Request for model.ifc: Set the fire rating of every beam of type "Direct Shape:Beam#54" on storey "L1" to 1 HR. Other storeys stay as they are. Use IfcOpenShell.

First a look at what the model holds.

```python
import ifcopenshell
import ifcopenshell.util.element

model = ifcopenshell.open("model.ifc")
print(model.schema)
storey = next(s for s in model.by_type("IfcBuildingStorey") if s.Name == "L1")
beams = [e for e in ifcopenshell.util.element.get_decomposition(storey) if e.is_a("IfcBeam")]
seen = {}
for e in beams:
    element_type = ifcopenshell.util.element.get_type(e)
    key = (element_type.Name if element_type != e and element_type else None, ifcopenshell.util.element.get_pset(e, "Pset_BeamCommon", "FireRating"))
    seen[key] = seen.get(key, 0) + 1
for (name, value), count in sorted(seen.items(), key=str):
    print(count, "x", name, "|", value)
```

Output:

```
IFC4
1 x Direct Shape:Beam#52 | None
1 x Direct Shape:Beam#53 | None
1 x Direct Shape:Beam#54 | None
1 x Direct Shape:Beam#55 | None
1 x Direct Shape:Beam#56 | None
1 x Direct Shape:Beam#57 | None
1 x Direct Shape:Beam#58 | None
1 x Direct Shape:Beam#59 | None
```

```python
import ifcopenshell
import ifcopenshell.api.pset
import ifcopenshell.util.element

model = ifcopenshell.open("model.ifc")

storey = next(s for s in model.by_type("IfcBuildingStorey") if s.Name == "L1")
beams = [e for e in ifcopenshell.util.element.get_decomposition(storey) if e.is_a("IfcBeam")]

count = 0
for e in beams:
    element_type = ifcopenshell.util.element.get_type(e)
    if element_type in (None, e) or element_type.Name != "Direct Shape:Beam#54":
        continue
    # add_pset returns the element's existing set when there is one.
    pset = ifcopenshell.api.pset.add_pset(model, product=e, name="Pset_BeamCommon")
    ifcopenshell.api.pset.edit_pset(model, pset=pset, properties={"FireRating": "1 HR"})
    count += 1

print(count, "beams updated")

model.write("model_v2.ifc")
```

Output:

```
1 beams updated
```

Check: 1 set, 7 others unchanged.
